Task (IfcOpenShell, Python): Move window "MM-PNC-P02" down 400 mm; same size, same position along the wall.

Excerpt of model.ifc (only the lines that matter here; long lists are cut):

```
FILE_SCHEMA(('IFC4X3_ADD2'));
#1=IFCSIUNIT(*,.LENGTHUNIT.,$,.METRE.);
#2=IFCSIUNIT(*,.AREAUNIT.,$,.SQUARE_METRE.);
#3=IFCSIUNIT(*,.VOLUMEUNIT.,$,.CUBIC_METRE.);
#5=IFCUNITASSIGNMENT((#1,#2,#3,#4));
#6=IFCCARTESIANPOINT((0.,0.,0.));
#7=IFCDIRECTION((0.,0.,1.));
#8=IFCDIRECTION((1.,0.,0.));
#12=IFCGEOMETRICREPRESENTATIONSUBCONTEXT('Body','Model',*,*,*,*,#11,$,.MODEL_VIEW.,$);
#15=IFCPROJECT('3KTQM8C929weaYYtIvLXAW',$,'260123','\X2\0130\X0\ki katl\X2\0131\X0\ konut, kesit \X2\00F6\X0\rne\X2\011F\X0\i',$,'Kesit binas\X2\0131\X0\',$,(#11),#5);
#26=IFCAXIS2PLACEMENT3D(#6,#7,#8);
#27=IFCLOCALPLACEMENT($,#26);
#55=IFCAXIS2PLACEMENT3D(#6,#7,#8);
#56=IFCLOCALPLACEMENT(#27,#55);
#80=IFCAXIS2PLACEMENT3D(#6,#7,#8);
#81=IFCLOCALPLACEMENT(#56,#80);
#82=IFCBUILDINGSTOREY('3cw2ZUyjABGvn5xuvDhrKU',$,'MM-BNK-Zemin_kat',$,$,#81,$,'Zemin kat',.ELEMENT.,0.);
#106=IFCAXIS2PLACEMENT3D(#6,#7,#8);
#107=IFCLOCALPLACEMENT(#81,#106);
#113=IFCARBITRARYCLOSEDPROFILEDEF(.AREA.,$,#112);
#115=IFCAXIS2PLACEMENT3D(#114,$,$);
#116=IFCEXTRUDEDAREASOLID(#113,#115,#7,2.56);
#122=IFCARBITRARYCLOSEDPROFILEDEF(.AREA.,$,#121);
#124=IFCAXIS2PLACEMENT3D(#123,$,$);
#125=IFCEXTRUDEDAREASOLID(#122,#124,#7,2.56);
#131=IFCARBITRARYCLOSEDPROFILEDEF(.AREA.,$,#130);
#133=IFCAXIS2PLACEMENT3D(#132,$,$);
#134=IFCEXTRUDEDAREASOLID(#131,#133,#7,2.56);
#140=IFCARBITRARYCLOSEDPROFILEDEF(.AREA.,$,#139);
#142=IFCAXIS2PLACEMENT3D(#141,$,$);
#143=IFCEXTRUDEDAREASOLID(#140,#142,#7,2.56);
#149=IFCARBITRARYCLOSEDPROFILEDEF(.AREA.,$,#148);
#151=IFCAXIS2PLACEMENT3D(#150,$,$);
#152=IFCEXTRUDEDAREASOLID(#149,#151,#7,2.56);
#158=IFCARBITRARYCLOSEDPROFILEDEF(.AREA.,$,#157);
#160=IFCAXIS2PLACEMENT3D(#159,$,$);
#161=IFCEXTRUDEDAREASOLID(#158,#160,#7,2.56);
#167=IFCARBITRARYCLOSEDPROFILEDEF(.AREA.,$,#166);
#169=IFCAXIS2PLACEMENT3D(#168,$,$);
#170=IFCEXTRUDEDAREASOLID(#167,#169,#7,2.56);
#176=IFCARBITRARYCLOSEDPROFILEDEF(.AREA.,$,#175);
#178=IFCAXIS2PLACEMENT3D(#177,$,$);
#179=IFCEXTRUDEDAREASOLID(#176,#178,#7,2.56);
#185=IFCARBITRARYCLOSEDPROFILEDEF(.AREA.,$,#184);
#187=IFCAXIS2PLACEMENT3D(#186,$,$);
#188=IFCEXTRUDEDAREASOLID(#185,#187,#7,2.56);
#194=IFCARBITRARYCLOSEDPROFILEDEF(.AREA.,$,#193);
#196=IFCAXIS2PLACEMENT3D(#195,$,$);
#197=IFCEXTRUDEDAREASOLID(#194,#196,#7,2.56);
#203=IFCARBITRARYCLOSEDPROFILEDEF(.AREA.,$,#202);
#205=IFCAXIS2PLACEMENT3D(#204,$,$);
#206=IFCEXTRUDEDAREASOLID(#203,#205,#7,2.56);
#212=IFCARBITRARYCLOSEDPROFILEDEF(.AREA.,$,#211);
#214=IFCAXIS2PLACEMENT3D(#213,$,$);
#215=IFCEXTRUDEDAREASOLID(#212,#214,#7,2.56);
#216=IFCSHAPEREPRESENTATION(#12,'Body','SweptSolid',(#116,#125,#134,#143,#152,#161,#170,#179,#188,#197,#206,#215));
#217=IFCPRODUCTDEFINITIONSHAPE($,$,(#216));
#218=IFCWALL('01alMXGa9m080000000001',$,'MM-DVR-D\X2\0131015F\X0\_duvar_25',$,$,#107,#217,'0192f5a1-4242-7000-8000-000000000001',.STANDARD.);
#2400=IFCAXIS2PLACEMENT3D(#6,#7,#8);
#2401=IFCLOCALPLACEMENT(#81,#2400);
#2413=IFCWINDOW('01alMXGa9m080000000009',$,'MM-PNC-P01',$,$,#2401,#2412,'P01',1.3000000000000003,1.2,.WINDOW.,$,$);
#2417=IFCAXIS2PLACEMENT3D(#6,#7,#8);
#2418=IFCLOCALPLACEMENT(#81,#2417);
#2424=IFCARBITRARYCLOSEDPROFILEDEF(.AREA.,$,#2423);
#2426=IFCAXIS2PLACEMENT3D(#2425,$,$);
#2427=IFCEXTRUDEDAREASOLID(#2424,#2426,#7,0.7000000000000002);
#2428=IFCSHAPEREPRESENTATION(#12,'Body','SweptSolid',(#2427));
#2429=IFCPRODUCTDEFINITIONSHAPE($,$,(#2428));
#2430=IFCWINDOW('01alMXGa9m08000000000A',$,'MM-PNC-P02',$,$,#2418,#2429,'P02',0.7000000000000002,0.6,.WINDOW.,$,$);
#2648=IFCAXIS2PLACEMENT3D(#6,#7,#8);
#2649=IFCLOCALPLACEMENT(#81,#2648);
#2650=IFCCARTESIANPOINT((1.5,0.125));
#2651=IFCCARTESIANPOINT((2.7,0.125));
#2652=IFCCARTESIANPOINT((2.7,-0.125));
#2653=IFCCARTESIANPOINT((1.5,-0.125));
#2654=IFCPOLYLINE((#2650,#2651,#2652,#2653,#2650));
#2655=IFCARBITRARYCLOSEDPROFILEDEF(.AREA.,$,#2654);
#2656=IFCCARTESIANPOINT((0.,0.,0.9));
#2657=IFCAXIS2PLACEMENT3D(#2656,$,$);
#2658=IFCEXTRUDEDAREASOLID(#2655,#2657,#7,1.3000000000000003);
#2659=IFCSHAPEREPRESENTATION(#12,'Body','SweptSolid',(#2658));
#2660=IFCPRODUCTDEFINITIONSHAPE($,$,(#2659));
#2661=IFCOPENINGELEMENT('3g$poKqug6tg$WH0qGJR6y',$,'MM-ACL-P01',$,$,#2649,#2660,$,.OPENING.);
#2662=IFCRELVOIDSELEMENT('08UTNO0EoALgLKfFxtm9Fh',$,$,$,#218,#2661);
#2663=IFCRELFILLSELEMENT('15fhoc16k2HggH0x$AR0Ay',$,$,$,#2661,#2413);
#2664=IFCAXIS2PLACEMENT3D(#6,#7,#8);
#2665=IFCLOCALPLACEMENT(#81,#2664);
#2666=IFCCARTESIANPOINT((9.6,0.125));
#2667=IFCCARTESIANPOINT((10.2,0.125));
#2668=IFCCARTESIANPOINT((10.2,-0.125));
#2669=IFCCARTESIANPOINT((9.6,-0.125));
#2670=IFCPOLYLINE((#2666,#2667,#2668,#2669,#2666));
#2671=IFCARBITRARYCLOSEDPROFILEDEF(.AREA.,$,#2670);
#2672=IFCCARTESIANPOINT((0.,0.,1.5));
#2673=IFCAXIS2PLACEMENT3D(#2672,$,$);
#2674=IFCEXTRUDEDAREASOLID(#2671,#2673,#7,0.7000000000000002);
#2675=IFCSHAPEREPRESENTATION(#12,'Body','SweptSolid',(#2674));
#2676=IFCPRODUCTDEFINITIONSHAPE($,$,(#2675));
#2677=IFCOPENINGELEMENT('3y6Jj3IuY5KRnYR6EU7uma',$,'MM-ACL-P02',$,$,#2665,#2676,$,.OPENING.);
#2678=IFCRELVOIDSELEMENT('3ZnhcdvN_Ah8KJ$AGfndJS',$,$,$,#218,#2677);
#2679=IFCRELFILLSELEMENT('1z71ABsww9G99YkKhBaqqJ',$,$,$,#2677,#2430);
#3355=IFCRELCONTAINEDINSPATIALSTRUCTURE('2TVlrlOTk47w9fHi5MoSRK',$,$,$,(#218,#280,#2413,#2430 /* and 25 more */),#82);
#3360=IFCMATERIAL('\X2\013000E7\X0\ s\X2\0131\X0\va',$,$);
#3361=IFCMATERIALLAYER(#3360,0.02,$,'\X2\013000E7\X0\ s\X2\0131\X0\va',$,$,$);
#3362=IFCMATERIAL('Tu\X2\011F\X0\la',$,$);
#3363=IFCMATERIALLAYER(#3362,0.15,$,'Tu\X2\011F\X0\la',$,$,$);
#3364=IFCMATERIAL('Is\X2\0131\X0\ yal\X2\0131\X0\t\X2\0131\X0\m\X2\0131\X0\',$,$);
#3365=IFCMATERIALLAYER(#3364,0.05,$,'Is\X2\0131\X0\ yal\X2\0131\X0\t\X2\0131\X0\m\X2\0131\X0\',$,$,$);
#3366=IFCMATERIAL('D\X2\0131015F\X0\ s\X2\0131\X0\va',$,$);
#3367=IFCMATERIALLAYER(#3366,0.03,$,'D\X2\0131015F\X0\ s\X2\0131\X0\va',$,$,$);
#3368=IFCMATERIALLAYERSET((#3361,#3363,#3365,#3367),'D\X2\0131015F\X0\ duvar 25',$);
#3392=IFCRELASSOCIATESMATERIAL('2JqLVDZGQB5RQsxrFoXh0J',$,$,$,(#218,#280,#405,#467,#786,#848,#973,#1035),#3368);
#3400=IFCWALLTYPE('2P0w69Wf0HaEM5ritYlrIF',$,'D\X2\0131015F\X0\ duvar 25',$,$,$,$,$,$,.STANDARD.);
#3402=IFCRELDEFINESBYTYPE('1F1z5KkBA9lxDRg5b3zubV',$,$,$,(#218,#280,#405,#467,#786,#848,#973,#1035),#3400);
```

```python
import numpy as np
import ifcopenshell
import ifcopenshell.api.geometry
import ifcopenshell.util.placement
import ifcopenshell.util.unit

model = ifcopenshell.open("model.ifc")
unit_scale = ifcopenshell.util.unit.calculate_unit_scale(model)

window = model.by_guid("01alMXGa9m08000000000A")
opening = window.FillsVoids[0].RelatingOpeningElement
dz = -0.4 / unit_scale

shift = np.array([0.0, 0.0, dz])
# The window is not placed relative to its opening, so move both.
for product in (opening, window):
    matrix = ifcopenshell.util.placement.get_local_placement(product.ObjectPlacement)
    matrix[:3, 3] += shift
    ifcopenshell.api.geometry.edit_object_placement(model, product=product, matrix=matrix, is_si=False)

print(f"moved by {dz * unit_scale:+.3f} m")

model.write("model_edited.ifc")
```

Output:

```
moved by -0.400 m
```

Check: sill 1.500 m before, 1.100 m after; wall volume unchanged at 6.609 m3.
